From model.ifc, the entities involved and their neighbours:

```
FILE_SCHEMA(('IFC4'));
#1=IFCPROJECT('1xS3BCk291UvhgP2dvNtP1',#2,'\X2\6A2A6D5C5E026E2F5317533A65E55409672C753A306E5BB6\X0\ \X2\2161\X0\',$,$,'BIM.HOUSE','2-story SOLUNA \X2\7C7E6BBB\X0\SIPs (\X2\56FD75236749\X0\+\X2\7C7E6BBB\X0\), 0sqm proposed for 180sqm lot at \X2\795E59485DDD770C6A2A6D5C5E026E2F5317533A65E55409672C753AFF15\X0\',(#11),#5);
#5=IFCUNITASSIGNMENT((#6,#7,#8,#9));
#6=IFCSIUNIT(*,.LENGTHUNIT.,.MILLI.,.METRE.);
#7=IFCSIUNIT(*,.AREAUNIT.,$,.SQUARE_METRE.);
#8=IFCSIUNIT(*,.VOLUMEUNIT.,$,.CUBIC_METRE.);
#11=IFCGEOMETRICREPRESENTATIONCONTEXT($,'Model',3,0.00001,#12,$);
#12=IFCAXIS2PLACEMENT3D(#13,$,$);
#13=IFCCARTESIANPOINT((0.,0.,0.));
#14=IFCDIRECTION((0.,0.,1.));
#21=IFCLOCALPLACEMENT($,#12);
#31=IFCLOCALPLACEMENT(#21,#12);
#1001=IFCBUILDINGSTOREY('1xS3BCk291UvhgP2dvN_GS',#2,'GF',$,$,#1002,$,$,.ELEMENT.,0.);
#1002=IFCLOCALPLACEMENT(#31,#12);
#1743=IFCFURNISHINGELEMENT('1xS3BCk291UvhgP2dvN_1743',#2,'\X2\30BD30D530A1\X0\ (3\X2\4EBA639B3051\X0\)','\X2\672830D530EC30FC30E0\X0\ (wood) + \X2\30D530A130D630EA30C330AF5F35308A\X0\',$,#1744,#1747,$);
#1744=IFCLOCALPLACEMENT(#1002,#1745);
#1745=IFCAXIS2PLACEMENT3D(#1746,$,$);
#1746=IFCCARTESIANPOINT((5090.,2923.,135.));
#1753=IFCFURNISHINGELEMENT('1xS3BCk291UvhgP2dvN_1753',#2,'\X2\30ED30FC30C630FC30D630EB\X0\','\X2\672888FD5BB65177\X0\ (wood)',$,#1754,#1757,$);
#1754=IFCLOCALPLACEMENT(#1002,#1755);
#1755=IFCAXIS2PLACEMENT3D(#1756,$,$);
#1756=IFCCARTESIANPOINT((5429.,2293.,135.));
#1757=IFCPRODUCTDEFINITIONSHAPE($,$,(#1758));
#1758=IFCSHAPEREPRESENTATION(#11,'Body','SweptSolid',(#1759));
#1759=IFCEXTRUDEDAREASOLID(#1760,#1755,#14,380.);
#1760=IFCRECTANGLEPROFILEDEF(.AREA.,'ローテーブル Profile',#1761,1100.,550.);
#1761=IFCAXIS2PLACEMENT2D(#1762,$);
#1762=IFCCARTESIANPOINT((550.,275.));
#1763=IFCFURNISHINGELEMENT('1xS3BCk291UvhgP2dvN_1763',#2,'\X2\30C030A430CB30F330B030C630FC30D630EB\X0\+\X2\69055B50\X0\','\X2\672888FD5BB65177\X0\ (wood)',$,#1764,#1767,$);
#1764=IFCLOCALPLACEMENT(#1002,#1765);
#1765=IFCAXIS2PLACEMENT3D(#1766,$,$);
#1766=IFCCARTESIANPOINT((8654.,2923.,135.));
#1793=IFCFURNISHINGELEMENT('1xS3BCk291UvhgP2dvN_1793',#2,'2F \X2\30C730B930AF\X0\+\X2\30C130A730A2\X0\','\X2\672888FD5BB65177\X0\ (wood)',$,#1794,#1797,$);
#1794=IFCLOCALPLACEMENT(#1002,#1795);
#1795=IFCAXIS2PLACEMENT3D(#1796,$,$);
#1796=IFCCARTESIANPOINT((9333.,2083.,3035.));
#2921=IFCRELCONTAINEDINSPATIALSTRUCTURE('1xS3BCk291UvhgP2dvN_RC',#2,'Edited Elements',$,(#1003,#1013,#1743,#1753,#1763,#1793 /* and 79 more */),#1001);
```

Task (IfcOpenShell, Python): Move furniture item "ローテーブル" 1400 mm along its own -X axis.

```python
import ifcopenshell
import ifcopenshell.api.geometry
import ifcopenshell.util.placement

model = ifcopenshell.open("model.ifc")

item = model.by_id(1753)
matrix = ifcopenshell.util.placement.get_local_placement(item.ObjectPlacement)
matrix[:3, 3] -= matrix[:3, 0] * 1400.0
ifcopenshell.api.geometry.edit_object_placement(model, product=item, matrix=matrix, is_si=False)

print(ifcopenshell.util.placement.get_local_placement(item.ObjectPlacement).round(3) + 0.0)

model.write("model-out.ifc")
```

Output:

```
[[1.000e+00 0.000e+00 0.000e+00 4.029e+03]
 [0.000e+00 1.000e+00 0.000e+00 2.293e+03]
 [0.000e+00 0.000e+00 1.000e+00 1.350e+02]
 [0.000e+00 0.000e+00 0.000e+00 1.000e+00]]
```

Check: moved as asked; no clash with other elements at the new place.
